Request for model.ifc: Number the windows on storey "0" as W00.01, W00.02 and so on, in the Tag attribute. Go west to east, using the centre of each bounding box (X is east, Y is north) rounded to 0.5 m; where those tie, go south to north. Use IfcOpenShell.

First a look at what the model holds.

```python
import ifcopenshell
import ifcopenshell.util.element
import ifcopenshell.util.placement

model = ifcopenshell.open("model.ifc")
print(model.schema)
storey = next(s for s in model.by_type("IfcBuildingStorey") if s.Name == "0")
windows = [e for e in ifcopenshell.util.element.get_decomposition(storey) if e.is_a("IfcWindow")]
for e in sorted(windows, key=lambda e: e.id()):
    origin = ifcopenshell.util.placement.get_local_placement(e.ObjectPlacement)[:3, 3]
    print(e.id(), e.Tag, e.Name, origin.round(2) + 0.0, sep=" | ")
```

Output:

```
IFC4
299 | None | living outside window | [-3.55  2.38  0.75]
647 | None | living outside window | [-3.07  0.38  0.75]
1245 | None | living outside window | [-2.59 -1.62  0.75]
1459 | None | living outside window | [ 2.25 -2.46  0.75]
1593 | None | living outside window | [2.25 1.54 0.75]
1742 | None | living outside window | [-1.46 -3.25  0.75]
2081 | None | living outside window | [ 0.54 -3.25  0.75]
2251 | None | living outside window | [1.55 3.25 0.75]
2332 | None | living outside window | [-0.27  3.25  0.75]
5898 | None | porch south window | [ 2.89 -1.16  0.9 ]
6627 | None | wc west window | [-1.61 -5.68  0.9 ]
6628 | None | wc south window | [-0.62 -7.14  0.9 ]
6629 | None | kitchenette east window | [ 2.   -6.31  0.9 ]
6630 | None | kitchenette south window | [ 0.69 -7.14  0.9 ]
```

```python
import ifcopenshell
import ifcopenshell.geom
import ifcopenshell.util.element
import ifcopenshell.util.shape

model = ifcopenshell.open("model.ifc")
settings = ifcopenshell.geom.settings()
settings.set("use-world-coords", True)


def centre(element):
    shape = ifcopenshell.geom.create_shape(settings, element)
    return ifcopenshell.util.shape.get_bbox_centroid(shape.geometry)


storey = next(s for s in model.by_type("IfcBuildingStorey") if s.Name == "0")
windows = [e for e in ifcopenshell.util.element.get_decomposition(storey) if e.is_a("IfcWindow")]

# Insertion points can sit at a corner or the storey origin, so sort by the geometry (in metres).
centres = {e: centre(e) for e in windows}
windows.sort(key=lambda e: (round(centres[e][0] / 0.5), centres[e][1]))

for i, e in enumerate(windows, start=1):
    number = f"W00.{i:02d}"
    e.Tag = number
    print(e.id(), number)

model.write("model_rev.ifc")
```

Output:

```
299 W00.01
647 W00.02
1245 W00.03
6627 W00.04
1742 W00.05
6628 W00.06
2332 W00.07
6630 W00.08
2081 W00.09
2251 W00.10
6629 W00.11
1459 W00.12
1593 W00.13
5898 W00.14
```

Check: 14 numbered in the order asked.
